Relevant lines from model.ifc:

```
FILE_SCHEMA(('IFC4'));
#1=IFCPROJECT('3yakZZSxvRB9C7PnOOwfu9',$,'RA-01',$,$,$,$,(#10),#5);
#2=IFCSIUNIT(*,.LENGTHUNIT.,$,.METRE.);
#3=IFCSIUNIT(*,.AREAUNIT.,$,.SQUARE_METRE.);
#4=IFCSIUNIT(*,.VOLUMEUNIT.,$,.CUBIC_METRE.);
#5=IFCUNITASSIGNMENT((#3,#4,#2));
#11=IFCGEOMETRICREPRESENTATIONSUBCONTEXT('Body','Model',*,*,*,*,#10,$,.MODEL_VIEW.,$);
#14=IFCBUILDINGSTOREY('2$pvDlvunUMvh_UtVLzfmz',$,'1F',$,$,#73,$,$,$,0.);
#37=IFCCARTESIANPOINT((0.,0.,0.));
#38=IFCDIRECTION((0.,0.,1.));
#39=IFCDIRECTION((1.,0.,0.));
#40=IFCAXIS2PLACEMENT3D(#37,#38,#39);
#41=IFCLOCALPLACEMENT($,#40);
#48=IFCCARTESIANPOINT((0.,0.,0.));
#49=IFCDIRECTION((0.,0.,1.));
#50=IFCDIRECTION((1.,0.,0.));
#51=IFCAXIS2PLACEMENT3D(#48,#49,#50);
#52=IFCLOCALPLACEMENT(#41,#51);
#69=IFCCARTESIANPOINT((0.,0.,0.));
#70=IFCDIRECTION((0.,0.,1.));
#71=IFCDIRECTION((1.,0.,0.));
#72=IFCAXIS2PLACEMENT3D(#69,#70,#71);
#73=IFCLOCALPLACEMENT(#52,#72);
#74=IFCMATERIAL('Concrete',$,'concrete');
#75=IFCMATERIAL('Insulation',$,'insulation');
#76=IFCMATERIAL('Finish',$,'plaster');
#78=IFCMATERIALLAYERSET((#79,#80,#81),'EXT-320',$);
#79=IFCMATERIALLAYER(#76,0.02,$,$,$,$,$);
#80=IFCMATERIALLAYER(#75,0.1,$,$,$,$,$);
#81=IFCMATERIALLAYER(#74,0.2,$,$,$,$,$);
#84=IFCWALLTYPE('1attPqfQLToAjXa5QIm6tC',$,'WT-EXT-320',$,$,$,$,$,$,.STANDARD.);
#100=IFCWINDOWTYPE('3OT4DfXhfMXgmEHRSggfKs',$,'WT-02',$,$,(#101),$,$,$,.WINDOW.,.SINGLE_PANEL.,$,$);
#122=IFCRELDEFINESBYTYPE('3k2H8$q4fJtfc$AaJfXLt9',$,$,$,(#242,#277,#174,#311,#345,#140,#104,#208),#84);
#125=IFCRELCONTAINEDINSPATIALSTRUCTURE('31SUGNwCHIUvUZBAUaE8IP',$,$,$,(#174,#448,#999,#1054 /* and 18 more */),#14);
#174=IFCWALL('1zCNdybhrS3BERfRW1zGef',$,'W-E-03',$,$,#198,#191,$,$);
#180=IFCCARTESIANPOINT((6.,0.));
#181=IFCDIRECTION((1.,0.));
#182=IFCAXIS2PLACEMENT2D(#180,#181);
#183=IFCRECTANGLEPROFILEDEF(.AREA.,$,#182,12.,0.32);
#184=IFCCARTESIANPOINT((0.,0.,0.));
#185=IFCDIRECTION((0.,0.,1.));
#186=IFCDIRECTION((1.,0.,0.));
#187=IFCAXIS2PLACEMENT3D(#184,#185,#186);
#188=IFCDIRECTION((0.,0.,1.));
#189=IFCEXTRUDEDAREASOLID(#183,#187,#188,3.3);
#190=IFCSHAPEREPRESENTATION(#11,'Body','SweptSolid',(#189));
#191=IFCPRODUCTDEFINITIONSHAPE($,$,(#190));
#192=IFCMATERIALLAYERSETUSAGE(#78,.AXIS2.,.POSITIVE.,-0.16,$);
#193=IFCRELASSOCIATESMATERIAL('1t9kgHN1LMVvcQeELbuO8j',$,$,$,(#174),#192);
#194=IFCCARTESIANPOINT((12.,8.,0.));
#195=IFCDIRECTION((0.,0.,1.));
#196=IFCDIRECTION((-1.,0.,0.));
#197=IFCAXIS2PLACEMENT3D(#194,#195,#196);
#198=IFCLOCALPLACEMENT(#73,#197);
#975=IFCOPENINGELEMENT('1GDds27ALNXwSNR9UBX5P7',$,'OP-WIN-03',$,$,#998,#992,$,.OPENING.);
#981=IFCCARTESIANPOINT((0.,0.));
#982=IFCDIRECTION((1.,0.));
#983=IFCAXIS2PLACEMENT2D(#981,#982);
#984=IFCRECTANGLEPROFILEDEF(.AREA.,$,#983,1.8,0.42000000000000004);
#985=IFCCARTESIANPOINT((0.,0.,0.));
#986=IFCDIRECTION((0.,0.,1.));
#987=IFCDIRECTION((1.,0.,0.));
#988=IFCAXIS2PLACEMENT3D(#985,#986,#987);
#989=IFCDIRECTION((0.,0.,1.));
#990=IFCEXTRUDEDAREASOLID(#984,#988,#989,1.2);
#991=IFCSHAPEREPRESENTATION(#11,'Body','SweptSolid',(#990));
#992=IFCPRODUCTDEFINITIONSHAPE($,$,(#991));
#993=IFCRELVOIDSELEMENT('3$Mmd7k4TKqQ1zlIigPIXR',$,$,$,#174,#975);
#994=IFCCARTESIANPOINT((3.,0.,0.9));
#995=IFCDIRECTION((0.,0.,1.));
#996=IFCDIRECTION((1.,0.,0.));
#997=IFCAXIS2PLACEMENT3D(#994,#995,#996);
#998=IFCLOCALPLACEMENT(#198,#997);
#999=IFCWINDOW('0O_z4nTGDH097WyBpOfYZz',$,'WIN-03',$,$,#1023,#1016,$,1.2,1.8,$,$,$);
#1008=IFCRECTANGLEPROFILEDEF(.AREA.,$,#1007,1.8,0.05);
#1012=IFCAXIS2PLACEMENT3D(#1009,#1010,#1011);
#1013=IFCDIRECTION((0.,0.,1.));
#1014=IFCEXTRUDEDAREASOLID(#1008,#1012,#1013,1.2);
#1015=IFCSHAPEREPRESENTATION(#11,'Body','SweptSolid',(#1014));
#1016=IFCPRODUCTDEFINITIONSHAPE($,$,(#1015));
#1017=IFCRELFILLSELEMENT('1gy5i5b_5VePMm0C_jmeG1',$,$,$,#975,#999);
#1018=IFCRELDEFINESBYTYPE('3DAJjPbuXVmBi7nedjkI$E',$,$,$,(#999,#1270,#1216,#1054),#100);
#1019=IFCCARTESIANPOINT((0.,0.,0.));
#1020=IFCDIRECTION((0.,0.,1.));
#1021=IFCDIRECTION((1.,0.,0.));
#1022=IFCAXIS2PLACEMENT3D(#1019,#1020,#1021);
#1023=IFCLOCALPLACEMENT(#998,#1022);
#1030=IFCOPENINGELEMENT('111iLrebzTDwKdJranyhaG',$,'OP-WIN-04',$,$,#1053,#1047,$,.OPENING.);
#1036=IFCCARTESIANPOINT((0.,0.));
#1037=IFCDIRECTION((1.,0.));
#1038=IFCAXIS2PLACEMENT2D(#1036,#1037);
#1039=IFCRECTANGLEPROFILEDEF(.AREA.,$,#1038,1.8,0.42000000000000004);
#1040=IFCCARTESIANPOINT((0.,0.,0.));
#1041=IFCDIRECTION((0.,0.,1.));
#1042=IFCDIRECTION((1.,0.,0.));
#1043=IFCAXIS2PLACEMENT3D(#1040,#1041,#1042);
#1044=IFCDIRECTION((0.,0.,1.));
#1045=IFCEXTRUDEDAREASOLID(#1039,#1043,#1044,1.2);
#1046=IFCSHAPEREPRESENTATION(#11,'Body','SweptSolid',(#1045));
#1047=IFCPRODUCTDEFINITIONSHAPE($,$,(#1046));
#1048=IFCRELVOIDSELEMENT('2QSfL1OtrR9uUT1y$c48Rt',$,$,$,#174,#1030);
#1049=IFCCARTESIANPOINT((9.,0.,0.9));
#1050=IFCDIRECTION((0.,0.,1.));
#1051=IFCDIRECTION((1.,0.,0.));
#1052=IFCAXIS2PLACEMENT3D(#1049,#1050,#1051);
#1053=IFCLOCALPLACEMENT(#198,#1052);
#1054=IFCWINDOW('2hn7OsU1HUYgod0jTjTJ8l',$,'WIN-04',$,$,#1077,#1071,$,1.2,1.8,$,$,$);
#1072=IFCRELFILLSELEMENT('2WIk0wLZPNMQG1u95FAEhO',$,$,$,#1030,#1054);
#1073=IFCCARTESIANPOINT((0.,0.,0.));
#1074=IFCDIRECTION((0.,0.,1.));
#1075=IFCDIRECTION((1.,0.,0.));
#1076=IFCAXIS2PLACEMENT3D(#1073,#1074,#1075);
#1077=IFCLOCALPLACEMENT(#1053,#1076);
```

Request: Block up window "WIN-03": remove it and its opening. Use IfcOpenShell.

```python
import ifcopenshell
import ifcopenshell.api.feature
import ifcopenshell.api.root
import ifcopenshell.geom
import ifcopenshell.util.shape

model = ifcopenshell.open("model.ifc")
settings = ifcopenshell.geom.settings()


def volume(element):
    """Net volume in cubic metres, openings subtracted."""
    shape = ifcopenshell.geom.create_shape(settings, element)
    return ifcopenshell.util.shape.get_volume(shape.geometry)


window = model.by_id(999)
opening = window.FillsVoids[0].RelatingOpeningElement
wall = opening.VoidsElements[0].RelatingBuildingElement
before = volume(wall)

ifcopenshell.api.root.remove_product(model, product=window)
ifcopenshell.api.feature.remove_feature(model, feature=opening)

after = volume(wall)

print(f"wall volume {before:.3f} -> {after:.3f} m3")

model.write("model_updated.ifc")
```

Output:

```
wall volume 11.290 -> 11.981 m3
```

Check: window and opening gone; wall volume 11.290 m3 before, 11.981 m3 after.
